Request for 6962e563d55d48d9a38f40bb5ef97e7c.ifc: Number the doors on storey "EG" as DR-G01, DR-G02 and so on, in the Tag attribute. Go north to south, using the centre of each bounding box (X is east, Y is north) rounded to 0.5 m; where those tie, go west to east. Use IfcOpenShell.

First a look at what the model holds.

```python
import ifcopenshell
import ifcopenshell.util.element
import ifcopenshell.util.placement

model = ifcopenshell.open("6962e563d55d48d9a38f40bb5ef97e7c.ifc")
print(model.schema)
storey = next(s for s in model.by_type("IfcBuildingStorey") if s.Name == "EG")
doors = [e for e in ifcopenshell.util.element.get_decomposition(storey) if e.is_a("IfcDoor")]
for e in sorted(doors, key=lambda e: e.id()):
    origin = ifcopenshell.util.placement.get_local_placement(e.ObjectPlacement)[:3, 3]
    print(e.id(), e.Tag, e.Name, origin.round(2) + 0.0, sep=" | ")
```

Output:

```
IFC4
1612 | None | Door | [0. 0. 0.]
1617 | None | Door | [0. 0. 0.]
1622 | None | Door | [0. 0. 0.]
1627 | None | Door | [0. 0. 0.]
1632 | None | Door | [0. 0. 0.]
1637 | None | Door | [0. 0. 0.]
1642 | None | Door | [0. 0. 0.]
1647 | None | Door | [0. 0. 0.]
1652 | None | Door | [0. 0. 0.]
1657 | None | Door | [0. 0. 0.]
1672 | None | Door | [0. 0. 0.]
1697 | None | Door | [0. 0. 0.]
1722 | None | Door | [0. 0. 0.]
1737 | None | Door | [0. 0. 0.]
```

```python
import ifcopenshell
import ifcopenshell.geom
import ifcopenshell.util.element
import ifcopenshell.util.shape

model = ifcopenshell.open("6962e563d55d48d9a38f40bb5ef97e7c.ifc")
settings = ifcopenshell.geom.settings()
settings.set("use-world-coords", True)


def centre(element):
    shape = ifcopenshell.geom.create_shape(settings, element)
    return ifcopenshell.util.shape.get_bbox_centroid(shape.geometry)


storey = next(s for s in model.by_type("IfcBuildingStorey") if s.Name == "EG")
doors = [e for e in ifcopenshell.util.element.get_decomposition(storey) if e.is_a("IfcDoor")]

# Insertion points can sit at a corner or the storey origin, so sort by the geometry (in metres).
centres = {e: centre(e) for e in doors}
doors.sort(key=lambda e: (-round(centres[e][1] / 0.5), centres[e][0]))

for i, e in enumerate(doors, start=1):
    number = f"DR-G{i:02d}"
    e.Tag = number
    print(e.id(), number)

model.write("6962e563d55d48d9a38f40bb5ef97e7c_updated.ifc")
```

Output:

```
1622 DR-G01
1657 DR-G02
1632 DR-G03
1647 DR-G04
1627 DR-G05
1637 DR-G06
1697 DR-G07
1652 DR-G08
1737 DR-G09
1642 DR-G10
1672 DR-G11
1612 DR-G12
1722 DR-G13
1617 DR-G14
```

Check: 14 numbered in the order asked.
